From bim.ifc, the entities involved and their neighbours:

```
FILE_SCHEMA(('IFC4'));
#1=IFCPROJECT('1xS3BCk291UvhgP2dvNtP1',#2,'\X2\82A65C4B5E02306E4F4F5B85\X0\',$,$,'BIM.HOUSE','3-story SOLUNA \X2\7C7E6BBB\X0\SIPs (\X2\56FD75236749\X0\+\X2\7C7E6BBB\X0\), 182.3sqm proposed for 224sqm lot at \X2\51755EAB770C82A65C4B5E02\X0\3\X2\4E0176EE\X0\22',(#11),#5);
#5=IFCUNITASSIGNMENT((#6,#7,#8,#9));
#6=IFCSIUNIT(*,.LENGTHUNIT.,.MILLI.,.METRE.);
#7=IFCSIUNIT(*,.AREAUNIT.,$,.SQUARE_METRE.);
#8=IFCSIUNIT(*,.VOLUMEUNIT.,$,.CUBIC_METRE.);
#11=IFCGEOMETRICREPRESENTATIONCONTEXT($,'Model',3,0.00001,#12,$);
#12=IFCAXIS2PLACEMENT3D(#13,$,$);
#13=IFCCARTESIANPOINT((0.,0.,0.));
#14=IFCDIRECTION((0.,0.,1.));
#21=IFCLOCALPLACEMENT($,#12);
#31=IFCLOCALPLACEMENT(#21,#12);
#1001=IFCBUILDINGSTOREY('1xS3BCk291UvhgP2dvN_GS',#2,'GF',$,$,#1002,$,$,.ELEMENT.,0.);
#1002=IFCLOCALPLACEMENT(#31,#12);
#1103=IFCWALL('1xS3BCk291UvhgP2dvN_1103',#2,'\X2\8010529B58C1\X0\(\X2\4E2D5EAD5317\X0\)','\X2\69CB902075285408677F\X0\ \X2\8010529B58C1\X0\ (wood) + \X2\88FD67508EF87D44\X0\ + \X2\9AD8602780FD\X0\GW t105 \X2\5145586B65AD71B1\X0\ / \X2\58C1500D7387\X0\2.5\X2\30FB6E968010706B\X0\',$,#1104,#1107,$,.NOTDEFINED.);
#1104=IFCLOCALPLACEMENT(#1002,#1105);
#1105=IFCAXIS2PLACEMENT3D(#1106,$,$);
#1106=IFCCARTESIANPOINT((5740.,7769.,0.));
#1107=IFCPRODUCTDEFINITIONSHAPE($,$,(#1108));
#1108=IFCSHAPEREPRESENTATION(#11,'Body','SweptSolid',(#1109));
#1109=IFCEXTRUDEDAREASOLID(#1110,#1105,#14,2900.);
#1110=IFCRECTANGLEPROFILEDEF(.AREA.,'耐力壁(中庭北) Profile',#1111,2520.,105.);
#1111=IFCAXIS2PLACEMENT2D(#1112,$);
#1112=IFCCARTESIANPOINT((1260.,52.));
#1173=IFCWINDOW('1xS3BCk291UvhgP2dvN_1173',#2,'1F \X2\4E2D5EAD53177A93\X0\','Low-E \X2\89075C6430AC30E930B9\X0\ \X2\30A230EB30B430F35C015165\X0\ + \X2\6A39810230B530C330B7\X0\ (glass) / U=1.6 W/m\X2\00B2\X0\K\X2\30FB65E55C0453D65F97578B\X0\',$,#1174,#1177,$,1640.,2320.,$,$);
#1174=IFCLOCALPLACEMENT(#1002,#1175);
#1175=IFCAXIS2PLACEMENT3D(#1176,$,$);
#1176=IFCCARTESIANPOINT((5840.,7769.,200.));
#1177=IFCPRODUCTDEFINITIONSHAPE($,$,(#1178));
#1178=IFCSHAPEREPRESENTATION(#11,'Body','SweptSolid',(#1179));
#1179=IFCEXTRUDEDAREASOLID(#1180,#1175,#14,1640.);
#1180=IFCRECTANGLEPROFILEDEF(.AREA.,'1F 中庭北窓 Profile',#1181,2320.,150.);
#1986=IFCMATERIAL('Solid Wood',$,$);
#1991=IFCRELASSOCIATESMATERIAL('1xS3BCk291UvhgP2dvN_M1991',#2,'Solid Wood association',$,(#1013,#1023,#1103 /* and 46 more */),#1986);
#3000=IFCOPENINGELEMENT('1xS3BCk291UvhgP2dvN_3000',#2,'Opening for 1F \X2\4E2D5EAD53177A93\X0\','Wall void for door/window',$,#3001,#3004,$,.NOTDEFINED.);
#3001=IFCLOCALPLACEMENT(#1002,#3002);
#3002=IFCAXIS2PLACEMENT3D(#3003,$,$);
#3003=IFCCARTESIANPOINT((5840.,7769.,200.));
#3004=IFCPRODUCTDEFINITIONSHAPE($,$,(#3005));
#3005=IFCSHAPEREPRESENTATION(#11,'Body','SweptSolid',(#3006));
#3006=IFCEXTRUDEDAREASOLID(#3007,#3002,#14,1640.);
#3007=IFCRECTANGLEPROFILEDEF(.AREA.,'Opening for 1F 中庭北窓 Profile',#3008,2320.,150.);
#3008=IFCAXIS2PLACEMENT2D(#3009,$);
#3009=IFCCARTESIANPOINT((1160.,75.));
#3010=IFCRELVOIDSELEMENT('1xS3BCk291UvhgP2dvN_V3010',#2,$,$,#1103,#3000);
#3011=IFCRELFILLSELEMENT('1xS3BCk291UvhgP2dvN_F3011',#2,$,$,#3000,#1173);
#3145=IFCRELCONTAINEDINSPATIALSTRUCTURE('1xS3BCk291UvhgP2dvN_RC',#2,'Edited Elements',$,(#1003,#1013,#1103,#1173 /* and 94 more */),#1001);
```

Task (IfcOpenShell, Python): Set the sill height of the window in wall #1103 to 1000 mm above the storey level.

```python
import numpy as np
import ifcopenshell
import ifcopenshell.api.geometry
import ifcopenshell.geom
import ifcopenshell.util.element
import ifcopenshell.util.placement
import ifcopenshell.util.shape
import ifcopenshell.util.unit

model = ifcopenshell.open("bim.ifc")
unit_scale = ifcopenshell.util.unit.calculate_unit_scale(model)

window = model.by_guid("1xS3BCk291UvhgP2dvN_1173")
opening = window.FillsVoids[0].RelatingOpeningElement
storey = ifcopenshell.util.element.get_container(window, ifc_class="IfcBuildingStorey")
level = ifcopenshell.util.placement.get_local_placement(storey.ObjectPlacement)[2, 3]

# The opening's origin need not be at the sill, so measure its lowest point.
shape = ifcopenshell.geom.create_shape(ifcopenshell.geom.settings(), opening)
bottom = ifcopenshell.util.shape.get_shape_bottom_elevation(shape, shape.geometry) / unit_scale
dz = level + 1 / unit_scale - bottom

shift = np.array([0.0, 0.0, dz])
# The window is not placed relative to its opening, so move both.
for product in (opening, window):
    matrix = ifcopenshell.util.placement.get_local_placement(product.ObjectPlacement)
    matrix[:3, 3] += shift
    ifcopenshell.api.geometry.edit_object_placement(model, product=product, matrix=matrix, is_si=False)

print(f"moved by {dz * unit_scale:+.3f} m")

model.write("bim_rev.ifc")
```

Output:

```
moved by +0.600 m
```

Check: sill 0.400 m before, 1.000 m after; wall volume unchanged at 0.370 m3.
